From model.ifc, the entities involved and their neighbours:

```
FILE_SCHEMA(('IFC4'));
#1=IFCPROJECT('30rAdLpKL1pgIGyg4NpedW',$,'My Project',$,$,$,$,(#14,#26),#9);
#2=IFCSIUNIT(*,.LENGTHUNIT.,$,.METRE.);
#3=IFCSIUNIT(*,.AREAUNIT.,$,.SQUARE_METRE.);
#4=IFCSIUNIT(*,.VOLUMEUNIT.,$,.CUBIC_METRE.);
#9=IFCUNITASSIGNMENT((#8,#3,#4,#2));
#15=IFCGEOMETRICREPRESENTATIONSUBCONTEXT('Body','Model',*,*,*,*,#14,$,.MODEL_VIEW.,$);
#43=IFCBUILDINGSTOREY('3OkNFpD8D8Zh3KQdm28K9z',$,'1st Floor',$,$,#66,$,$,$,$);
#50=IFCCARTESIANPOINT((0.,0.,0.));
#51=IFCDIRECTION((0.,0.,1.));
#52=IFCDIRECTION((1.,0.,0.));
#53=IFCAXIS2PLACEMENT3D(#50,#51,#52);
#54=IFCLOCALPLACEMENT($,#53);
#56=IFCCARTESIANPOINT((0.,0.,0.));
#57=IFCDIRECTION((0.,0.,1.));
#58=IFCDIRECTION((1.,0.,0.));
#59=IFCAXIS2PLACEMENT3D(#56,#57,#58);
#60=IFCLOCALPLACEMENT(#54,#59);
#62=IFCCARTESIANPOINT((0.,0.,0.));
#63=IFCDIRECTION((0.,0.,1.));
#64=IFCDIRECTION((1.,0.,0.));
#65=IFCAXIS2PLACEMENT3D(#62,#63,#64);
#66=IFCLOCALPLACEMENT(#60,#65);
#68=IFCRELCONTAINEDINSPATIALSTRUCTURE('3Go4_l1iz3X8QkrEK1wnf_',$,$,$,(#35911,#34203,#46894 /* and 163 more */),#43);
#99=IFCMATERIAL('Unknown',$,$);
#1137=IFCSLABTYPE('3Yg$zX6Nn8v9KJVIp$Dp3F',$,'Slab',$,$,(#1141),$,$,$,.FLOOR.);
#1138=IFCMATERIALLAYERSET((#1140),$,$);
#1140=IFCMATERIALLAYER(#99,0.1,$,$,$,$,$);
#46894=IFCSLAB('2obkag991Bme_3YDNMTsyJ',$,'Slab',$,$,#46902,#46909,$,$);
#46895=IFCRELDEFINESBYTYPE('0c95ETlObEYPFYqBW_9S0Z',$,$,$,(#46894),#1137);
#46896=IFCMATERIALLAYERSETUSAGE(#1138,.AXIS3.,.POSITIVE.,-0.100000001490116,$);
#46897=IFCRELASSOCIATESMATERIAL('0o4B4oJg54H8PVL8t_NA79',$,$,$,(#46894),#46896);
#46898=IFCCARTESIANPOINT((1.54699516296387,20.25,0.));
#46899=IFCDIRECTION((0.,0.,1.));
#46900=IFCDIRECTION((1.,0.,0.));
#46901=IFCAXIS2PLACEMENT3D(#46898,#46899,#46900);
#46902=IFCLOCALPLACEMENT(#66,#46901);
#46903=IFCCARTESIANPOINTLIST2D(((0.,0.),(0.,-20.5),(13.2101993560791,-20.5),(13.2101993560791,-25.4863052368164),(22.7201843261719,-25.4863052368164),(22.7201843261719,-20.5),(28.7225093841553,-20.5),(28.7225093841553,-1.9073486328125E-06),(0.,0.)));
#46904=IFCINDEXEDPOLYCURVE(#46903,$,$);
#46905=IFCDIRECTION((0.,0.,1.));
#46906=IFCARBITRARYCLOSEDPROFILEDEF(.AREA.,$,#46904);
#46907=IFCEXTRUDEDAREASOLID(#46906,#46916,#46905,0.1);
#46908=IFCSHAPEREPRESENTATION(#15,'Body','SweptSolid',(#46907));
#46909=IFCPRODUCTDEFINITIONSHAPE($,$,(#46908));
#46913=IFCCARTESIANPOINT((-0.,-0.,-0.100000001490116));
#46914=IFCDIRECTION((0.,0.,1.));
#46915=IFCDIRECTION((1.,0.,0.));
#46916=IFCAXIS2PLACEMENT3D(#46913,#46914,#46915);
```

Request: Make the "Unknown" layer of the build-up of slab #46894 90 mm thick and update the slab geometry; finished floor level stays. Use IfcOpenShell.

```python
import ifcopenshell
import ifcopenshell.util.element
import ifcopenshell.util.representation
import ifcopenshell.util.unit

model = ifcopenshell.open("model.ifc")
unit_scale = ifcopenshell.util.unit.calculate_unit_scale(model)

layer_set = model.by_id(1138)
layer = next(l for l in layer_set.MaterialLayers if l.Material and l.Material.Name == "Unknown")
change = 0.09 / unit_scale - layer.LayerThickness
layer.LayerThickness += change

# Geometry does not follow the layer set by itself.
slabs = [e for e in ifcopenshell.util.element.get_elements_by_material(model, layer_set) if e.is_a("IfcSlab")]
for slab in sorted(slabs, key=lambda e: e.id()):
    body = ifcopenshell.util.representation.get_representation(slab, "Model", "Body")
    solid = body.Items[0]
    old_depth = solid.Depth
    solid.Depth += change
    # Extruded upwards: lower the start of the extrusion so the top stays.
    x, y, z = solid.Position.Location.Coordinates
    solid.Position.Location = model.createIfcCartesianPoint((x, y, z - change))
    print(slab.id(), f"{old_depth:g} -> {solid.Depth:g}")

# The layers are counted up from the underside, which has moved.
for usage in {ifcopenshell.util.element.get_material(slab) for slab in slabs}:
    usage.OffsetFromReferenceLine -= change

model.write("model_v2.ifc")
```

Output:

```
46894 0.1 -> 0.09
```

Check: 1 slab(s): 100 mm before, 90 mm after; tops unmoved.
